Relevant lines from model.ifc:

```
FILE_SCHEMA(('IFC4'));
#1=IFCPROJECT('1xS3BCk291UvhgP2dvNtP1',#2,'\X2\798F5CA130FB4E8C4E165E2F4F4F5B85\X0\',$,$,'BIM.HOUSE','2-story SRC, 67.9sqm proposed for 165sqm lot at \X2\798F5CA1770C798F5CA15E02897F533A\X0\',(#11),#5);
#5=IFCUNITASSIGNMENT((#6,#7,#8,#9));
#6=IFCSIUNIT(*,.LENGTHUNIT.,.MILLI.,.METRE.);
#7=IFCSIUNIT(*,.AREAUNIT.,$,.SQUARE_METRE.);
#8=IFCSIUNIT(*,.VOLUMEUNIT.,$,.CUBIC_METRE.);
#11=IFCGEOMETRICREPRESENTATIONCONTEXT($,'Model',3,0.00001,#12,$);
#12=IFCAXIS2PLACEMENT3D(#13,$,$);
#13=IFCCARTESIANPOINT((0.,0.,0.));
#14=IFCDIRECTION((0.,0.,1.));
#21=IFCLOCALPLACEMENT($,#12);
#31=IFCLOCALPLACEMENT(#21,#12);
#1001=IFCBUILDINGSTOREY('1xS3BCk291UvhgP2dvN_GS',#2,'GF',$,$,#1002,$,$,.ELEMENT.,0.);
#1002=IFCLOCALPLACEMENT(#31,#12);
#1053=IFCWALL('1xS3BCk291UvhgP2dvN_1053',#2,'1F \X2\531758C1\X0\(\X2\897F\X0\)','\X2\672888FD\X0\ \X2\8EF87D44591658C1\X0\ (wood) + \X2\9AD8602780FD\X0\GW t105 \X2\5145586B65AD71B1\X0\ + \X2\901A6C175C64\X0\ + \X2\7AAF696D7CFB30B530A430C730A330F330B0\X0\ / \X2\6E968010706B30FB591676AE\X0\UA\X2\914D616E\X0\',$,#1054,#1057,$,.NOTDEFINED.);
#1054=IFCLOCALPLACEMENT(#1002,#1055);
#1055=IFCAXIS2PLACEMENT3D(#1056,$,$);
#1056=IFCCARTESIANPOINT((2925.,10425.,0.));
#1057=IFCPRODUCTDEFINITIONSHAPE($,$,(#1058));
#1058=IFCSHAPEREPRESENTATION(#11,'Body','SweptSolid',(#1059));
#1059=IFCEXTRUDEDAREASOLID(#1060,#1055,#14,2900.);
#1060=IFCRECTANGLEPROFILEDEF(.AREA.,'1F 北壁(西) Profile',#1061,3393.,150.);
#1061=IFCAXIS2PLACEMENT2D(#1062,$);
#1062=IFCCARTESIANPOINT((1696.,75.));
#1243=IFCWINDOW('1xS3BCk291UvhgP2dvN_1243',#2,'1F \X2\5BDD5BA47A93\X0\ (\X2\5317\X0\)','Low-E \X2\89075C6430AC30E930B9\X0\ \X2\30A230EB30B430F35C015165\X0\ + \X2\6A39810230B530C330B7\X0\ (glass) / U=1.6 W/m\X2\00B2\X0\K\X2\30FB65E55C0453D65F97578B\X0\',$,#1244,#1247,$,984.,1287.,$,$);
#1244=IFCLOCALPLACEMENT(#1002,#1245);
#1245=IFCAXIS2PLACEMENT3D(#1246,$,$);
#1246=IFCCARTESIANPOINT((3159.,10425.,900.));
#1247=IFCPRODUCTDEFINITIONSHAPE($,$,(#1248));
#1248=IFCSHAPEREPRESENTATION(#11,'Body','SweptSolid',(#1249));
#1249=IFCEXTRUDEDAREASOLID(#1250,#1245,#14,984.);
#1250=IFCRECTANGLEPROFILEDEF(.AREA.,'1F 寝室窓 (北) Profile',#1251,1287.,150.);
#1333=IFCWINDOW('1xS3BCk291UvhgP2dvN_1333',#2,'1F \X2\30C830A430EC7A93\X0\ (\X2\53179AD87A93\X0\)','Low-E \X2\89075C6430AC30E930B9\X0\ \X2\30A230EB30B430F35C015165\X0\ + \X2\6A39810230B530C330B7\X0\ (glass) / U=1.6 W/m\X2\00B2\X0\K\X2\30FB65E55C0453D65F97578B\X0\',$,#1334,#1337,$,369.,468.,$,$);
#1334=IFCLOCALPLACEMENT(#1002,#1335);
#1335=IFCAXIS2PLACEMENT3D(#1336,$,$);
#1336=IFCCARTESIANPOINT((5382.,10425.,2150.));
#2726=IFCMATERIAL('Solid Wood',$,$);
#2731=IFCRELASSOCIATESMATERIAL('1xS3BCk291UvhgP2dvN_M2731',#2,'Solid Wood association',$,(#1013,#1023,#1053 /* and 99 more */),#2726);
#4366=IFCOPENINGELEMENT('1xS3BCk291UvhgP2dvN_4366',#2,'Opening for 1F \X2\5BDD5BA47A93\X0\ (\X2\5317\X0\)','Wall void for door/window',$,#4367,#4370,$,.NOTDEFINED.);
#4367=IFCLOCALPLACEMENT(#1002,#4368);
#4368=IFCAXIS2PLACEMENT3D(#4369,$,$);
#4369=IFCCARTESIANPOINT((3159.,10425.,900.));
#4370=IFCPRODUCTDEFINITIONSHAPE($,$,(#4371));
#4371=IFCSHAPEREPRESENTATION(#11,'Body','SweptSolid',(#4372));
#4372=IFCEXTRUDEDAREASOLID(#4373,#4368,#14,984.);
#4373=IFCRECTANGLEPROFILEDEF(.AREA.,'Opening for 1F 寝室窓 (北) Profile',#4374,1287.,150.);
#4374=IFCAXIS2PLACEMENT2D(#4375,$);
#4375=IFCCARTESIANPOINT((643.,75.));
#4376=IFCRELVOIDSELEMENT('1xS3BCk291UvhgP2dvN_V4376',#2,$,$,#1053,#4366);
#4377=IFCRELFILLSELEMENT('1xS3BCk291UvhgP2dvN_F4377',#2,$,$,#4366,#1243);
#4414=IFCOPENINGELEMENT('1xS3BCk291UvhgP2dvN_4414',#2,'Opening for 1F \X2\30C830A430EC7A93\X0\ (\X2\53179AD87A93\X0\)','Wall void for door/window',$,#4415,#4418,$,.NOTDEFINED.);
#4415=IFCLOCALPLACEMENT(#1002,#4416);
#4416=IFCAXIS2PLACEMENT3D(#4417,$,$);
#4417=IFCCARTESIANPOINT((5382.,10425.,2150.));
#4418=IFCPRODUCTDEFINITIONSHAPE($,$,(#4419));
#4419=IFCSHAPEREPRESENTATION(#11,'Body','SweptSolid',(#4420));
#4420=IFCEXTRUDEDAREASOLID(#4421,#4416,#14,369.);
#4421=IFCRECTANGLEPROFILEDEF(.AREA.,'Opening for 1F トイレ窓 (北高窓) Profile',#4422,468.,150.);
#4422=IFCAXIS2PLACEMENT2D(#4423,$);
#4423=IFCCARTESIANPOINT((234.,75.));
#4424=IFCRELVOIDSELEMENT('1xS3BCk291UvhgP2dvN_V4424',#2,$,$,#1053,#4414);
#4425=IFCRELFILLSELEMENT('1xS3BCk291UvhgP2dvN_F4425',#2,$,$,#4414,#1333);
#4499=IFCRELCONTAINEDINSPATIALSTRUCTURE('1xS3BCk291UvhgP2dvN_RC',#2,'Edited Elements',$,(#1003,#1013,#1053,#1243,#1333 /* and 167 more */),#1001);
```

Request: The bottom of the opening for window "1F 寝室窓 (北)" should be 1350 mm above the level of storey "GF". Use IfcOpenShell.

```python
import numpy as np
import ifcopenshell
import ifcopenshell.api.geometry
import ifcopenshell.geom
import ifcopenshell.util.element
import ifcopenshell.util.placement
import ifcopenshell.util.shape
import ifcopenshell.util.unit

model = ifcopenshell.open("model.ifc")
unit_scale = ifcopenshell.util.unit.calculate_unit_scale(model)

window = model.by_guid("1xS3BCk291UvhgP2dvN_1243")
opening = window.FillsVoids[0].RelatingOpeningElement
storey = ifcopenshell.util.element.get_container(window, ifc_class="IfcBuildingStorey")
level = ifcopenshell.util.placement.get_local_placement(storey.ObjectPlacement)[2, 3]

# The opening's origin need not be at the sill, so measure its lowest point.
shape = ifcopenshell.geom.create_shape(ifcopenshell.geom.settings(), opening)
bottom = ifcopenshell.util.shape.get_shape_bottom_elevation(shape, shape.geometry) / unit_scale
dz = level + 1.35 / unit_scale - bottom

shift = np.array([0.0, 0.0, dz])
# The window is not placed relative to its opening, so move both.
for product in (opening, window):
    matrix = ifcopenshell.util.placement.get_local_placement(product.ObjectPlacement)
    matrix[:3, 3] += shift
    ifcopenshell.api.geometry.edit_object_placement(model, product=product, matrix=matrix, is_si=False)

print(f"moved by {dz * unit_scale:+.3f} m")

model.write("model_rev.ifc")
```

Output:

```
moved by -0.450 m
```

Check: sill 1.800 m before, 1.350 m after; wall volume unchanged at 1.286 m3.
